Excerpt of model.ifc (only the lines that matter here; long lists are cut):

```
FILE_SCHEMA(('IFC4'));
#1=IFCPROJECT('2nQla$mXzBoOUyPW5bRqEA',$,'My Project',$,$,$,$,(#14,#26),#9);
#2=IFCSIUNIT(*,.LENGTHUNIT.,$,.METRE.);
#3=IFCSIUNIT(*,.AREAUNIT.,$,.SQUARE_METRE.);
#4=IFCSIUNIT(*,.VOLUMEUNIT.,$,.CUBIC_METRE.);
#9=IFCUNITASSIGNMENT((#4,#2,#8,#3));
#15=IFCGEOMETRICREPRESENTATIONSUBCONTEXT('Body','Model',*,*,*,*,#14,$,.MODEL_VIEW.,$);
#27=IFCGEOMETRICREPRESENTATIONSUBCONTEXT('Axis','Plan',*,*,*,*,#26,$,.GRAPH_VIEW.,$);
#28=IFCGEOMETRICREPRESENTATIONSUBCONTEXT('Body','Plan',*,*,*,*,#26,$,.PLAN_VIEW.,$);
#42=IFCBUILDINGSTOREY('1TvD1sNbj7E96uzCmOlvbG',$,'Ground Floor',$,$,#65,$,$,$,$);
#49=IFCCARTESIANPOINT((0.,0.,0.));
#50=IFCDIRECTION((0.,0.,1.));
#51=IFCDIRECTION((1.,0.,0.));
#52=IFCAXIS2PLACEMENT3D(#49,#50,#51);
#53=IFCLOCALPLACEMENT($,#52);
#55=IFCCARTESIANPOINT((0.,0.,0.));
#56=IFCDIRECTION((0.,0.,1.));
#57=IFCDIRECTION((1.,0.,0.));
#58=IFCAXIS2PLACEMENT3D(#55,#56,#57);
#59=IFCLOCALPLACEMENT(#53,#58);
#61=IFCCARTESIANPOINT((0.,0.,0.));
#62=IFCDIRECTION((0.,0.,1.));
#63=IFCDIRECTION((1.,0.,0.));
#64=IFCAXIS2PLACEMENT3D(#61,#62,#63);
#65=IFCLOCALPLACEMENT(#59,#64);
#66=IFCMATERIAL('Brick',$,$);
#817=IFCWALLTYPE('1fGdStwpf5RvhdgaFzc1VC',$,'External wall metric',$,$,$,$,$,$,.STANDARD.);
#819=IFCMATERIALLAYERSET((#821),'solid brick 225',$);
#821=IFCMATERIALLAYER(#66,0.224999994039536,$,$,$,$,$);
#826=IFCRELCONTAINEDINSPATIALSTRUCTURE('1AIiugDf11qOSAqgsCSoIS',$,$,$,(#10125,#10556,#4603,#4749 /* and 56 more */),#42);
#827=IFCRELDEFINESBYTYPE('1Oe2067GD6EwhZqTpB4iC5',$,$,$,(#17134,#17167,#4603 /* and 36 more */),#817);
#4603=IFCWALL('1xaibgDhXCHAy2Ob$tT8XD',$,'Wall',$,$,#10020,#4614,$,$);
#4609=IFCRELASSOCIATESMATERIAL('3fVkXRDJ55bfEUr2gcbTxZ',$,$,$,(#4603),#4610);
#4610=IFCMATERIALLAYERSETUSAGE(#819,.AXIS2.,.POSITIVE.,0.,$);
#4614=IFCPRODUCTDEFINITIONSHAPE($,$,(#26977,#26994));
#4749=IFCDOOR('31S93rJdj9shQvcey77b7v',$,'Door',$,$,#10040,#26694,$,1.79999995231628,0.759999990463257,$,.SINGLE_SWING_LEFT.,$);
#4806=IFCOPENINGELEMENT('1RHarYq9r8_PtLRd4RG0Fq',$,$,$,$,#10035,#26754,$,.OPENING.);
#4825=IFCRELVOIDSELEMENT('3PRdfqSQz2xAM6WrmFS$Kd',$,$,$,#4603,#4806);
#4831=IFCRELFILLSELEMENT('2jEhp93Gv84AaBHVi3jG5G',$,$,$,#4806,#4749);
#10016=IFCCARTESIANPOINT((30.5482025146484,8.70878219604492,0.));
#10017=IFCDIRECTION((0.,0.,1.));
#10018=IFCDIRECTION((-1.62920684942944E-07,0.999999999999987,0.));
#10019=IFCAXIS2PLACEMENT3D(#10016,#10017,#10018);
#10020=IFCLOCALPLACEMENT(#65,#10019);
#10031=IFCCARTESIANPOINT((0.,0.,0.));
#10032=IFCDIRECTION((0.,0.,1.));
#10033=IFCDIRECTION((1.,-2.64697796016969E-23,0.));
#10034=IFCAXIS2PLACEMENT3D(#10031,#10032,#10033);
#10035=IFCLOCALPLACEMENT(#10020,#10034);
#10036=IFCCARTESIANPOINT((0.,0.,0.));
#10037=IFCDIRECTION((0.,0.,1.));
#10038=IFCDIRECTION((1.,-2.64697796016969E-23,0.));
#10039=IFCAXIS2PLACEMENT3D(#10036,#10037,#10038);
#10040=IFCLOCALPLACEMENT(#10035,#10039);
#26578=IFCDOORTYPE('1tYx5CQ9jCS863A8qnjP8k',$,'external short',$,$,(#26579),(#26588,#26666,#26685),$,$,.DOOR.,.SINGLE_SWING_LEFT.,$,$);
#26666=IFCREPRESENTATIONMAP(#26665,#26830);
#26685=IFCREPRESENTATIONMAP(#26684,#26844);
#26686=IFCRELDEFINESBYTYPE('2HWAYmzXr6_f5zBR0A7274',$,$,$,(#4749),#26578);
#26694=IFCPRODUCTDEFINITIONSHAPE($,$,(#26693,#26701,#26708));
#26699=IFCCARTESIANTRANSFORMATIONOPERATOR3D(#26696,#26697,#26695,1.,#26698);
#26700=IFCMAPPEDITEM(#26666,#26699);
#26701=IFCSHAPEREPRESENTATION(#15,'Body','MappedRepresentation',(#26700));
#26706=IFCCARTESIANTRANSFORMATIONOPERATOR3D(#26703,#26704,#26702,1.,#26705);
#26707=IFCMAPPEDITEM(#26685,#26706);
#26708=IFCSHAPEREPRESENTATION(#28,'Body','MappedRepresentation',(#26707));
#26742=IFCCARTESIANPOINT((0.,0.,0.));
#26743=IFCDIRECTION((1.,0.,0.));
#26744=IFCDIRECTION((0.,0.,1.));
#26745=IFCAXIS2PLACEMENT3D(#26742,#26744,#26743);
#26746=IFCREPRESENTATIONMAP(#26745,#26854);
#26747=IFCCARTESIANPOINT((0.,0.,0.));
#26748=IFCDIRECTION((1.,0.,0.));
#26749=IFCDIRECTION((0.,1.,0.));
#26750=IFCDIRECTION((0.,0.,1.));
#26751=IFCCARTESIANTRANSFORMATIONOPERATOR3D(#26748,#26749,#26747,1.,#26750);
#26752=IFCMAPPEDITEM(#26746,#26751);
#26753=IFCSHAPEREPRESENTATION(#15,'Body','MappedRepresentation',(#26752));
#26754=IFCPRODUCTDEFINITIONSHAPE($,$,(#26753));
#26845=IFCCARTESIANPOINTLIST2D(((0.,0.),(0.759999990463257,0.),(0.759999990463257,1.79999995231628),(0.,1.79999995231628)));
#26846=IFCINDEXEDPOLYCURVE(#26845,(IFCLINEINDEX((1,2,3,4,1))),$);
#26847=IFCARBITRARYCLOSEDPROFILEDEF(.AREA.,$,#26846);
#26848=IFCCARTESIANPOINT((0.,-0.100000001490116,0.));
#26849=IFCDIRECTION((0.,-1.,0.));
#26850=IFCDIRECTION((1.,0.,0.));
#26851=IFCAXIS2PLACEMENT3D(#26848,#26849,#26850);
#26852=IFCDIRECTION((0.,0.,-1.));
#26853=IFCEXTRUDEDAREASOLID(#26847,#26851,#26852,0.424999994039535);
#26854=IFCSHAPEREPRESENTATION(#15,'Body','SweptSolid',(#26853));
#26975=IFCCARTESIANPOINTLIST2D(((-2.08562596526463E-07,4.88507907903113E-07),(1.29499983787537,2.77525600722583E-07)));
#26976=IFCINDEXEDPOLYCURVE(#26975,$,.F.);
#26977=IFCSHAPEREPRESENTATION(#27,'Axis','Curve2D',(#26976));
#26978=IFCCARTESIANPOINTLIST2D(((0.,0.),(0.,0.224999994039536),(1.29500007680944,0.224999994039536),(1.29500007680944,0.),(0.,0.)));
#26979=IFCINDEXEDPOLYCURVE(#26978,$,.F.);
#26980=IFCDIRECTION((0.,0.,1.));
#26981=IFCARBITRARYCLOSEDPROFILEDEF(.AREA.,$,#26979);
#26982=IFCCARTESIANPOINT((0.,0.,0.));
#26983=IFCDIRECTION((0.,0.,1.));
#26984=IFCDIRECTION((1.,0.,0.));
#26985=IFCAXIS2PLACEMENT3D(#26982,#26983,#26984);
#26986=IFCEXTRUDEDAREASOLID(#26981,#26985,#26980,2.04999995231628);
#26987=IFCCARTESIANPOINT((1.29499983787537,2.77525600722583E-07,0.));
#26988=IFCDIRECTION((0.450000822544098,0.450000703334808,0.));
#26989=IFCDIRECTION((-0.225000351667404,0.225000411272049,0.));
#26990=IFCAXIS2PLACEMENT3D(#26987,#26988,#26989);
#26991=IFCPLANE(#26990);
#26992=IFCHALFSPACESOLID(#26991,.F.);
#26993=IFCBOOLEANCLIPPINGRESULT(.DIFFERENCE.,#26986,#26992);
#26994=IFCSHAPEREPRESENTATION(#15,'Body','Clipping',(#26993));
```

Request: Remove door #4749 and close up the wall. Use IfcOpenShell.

```python
import ifcopenshell
import ifcopenshell.api.feature
import ifcopenshell.api.root
import ifcopenshell.geom
import ifcopenshell.util.shape

model = ifcopenshell.open("model.ifc")
settings = ifcopenshell.geom.settings()


def volume(element):
    """Net volume in cubic metres, openings subtracted."""
    shape = ifcopenshell.geom.create_shape(settings, element)
    return ifcopenshell.util.shape.get_volume(shape.geometry)


door = model.by_guid("31S93rJdj9shQvcey77b7v")
opening = door.FillsVoids[0].RelatingOpeningElement
wall = opening.VoidsElements[0].RelatingBuildingElement
before = volume(wall)

ifcopenshell.api.root.remove_product(model, product=door)
ifcopenshell.api.feature.remove_feature(model, feature=opening)

after = volume(wall)

print(f"wall volume {before:.3f} -> {after:.3f} m3")

model.write("model-out.ifc")
```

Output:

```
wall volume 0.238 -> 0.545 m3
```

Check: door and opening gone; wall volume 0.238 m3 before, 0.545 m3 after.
